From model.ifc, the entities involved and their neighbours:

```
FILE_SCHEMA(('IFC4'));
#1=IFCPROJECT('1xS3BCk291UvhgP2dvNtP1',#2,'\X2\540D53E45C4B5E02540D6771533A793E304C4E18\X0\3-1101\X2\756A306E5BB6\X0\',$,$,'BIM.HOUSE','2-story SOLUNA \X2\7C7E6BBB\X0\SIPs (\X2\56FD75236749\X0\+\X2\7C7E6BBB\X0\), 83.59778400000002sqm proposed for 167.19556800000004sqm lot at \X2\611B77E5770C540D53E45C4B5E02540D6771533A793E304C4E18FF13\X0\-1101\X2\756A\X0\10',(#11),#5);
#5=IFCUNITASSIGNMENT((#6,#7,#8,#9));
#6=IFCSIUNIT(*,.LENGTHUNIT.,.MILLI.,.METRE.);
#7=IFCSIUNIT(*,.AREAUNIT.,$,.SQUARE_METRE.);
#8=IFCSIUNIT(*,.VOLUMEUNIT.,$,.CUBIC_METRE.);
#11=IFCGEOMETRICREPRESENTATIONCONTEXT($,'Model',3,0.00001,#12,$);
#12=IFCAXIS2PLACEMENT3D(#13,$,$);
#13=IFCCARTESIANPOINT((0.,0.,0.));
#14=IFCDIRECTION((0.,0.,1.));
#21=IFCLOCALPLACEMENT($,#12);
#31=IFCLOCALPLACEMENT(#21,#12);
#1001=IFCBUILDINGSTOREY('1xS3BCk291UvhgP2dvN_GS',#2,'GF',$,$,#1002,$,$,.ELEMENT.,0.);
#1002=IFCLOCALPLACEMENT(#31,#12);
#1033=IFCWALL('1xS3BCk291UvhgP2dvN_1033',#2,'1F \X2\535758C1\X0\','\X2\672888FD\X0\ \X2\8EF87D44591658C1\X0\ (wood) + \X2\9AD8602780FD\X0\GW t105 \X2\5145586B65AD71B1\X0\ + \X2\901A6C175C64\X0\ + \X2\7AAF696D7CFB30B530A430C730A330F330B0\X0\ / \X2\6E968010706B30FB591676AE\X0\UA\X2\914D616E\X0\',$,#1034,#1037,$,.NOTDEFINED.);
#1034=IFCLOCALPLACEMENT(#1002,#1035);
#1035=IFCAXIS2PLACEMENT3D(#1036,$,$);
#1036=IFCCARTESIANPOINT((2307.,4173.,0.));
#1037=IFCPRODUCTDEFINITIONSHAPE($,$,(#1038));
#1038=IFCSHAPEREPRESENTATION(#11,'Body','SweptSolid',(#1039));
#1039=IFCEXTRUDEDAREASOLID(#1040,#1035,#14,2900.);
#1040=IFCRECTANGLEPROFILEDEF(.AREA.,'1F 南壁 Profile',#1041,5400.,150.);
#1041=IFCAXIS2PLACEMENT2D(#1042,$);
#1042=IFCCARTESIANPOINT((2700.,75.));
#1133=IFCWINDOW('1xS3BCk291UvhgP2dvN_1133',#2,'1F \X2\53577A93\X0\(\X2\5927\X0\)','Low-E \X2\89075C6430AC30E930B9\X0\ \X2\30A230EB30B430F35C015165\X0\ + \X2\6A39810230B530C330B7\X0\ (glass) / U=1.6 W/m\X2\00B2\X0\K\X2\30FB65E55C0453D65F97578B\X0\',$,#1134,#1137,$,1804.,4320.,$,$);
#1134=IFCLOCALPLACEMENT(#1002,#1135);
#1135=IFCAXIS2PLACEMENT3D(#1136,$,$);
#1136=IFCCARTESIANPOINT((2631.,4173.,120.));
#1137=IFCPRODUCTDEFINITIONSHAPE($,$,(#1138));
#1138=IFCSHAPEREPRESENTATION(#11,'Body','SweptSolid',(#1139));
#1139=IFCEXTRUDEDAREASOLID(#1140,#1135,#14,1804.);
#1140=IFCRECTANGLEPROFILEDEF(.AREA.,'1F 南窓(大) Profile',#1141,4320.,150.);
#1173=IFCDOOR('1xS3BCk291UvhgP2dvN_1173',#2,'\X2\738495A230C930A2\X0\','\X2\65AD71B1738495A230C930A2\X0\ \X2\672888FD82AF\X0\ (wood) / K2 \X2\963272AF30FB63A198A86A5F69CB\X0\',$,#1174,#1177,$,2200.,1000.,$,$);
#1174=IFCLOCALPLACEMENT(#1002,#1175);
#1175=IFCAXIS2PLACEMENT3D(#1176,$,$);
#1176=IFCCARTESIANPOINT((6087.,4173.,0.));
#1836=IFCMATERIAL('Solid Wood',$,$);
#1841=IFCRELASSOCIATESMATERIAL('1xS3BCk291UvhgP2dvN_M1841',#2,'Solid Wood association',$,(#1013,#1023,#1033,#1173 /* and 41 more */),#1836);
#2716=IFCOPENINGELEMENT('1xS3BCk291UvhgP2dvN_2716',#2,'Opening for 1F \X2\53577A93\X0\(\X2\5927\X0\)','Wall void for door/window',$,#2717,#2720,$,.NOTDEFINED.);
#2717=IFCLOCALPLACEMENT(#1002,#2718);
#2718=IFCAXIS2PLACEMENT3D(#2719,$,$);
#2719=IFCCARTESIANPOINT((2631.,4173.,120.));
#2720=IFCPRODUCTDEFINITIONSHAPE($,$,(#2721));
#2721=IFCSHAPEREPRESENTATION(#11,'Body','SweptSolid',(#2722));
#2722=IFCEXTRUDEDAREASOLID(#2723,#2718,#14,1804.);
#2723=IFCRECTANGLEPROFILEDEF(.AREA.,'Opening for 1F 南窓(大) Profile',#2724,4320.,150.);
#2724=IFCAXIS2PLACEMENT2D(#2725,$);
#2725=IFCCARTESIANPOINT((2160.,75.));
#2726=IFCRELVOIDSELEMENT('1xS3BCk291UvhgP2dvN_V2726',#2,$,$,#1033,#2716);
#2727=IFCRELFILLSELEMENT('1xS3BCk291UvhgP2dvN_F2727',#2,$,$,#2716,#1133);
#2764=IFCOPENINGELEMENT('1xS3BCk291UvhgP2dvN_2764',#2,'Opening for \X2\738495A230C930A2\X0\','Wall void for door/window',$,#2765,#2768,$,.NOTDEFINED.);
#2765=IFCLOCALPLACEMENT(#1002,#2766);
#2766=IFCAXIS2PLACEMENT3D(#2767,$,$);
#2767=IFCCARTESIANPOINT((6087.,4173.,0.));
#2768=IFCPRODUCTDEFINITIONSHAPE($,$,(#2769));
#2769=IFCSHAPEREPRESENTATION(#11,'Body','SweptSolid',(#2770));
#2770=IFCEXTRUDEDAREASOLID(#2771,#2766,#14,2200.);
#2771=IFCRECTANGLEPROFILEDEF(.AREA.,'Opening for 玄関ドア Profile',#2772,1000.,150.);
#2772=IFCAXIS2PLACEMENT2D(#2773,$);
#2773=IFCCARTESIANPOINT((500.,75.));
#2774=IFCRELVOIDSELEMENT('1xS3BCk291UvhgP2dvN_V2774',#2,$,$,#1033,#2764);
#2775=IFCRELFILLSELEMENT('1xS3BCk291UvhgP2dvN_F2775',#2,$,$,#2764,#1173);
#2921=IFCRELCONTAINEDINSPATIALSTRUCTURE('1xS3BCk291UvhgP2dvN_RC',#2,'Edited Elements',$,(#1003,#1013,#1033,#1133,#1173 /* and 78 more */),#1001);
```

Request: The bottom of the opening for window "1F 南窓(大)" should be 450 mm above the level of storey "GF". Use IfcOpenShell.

```python
import numpy as np
import ifcopenshell
import ifcopenshell.api.geometry
import ifcopenshell.geom
import ifcopenshell.util.element
import ifcopenshell.util.placement
import ifcopenshell.util.shape
import ifcopenshell.util.unit

model = ifcopenshell.open("model.ifc")
unit_scale = ifcopenshell.util.unit.calculate_unit_scale(model)

window = model.by_id(1133)
opening = window.FillsVoids[0].RelatingOpeningElement
storey = ifcopenshell.util.element.get_container(window, ifc_class="IfcBuildingStorey")
level = ifcopenshell.util.placement.get_local_placement(storey.ObjectPlacement)[2, 3]

# The opening's origin need not be at the sill, so measure its lowest point.
shape = ifcopenshell.geom.create_shape(ifcopenshell.geom.settings(), opening)
bottom = ifcopenshell.util.shape.get_shape_bottom_elevation(shape, shape.geometry) / unit_scale
dz = level + 0.45 / unit_scale - bottom

shift = np.array([0.0, 0.0, dz])
# The window is not placed relative to its opening, so move both.
for product in (opening, window):
    matrix = ifcopenshell.util.placement.get_local_placement(product.ObjectPlacement)
    matrix[:3, 3] += shift
    ifcopenshell.api.geometry.edit_object_placement(model, product=product, matrix=matrix, is_si=False)

print(f"moved by {dz * unit_scale:+.3f} m")

model.write("model_rev.ifc")
```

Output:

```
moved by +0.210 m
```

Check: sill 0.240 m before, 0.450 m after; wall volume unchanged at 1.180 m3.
